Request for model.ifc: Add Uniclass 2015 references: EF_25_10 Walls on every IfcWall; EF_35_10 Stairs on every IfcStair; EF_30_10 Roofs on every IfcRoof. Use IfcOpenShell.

First a look at what the model holds.

```python
import ifcopenshell

model = ifcopenshell.open("model.ifc")
print(model.schema)
print("classifications:", [c.Name for c in model.by_type("IfcClassification")])
for ifc_class in ("IfcDoor", "IfcRoof", "IfcStair", "IfcWall", "IfcWindow"):
    print(ifc_class, len(model.by_type(ifc_class)))
```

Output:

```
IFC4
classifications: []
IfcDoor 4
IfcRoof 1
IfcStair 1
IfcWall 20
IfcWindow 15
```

```python
import ifcopenshell
import ifcopenshell.api.classification

model = ifcopenshell.open("model.ifc")

system = ifcopenshell.api.classification.add_classification(model, classification="Uniclass 2015")

codes = {
    "IfcWall": ("EF_25_10", "Walls"),
    "IfcStair": ("EF_35_10", "Stairs"),
    "IfcRoof": ("EF_30_10", "Roofs"),
}
for ifc_class, (code, name) in codes.items():
    products = model.by_type(ifc_class)
    ifcopenshell.api.classification.add_reference(
        model, products=products, classification=system, identification=code, name=name
    )
    print(code, len(products))

model.write("model_updated.ifc")
```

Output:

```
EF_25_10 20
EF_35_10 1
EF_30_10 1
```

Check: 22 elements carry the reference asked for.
